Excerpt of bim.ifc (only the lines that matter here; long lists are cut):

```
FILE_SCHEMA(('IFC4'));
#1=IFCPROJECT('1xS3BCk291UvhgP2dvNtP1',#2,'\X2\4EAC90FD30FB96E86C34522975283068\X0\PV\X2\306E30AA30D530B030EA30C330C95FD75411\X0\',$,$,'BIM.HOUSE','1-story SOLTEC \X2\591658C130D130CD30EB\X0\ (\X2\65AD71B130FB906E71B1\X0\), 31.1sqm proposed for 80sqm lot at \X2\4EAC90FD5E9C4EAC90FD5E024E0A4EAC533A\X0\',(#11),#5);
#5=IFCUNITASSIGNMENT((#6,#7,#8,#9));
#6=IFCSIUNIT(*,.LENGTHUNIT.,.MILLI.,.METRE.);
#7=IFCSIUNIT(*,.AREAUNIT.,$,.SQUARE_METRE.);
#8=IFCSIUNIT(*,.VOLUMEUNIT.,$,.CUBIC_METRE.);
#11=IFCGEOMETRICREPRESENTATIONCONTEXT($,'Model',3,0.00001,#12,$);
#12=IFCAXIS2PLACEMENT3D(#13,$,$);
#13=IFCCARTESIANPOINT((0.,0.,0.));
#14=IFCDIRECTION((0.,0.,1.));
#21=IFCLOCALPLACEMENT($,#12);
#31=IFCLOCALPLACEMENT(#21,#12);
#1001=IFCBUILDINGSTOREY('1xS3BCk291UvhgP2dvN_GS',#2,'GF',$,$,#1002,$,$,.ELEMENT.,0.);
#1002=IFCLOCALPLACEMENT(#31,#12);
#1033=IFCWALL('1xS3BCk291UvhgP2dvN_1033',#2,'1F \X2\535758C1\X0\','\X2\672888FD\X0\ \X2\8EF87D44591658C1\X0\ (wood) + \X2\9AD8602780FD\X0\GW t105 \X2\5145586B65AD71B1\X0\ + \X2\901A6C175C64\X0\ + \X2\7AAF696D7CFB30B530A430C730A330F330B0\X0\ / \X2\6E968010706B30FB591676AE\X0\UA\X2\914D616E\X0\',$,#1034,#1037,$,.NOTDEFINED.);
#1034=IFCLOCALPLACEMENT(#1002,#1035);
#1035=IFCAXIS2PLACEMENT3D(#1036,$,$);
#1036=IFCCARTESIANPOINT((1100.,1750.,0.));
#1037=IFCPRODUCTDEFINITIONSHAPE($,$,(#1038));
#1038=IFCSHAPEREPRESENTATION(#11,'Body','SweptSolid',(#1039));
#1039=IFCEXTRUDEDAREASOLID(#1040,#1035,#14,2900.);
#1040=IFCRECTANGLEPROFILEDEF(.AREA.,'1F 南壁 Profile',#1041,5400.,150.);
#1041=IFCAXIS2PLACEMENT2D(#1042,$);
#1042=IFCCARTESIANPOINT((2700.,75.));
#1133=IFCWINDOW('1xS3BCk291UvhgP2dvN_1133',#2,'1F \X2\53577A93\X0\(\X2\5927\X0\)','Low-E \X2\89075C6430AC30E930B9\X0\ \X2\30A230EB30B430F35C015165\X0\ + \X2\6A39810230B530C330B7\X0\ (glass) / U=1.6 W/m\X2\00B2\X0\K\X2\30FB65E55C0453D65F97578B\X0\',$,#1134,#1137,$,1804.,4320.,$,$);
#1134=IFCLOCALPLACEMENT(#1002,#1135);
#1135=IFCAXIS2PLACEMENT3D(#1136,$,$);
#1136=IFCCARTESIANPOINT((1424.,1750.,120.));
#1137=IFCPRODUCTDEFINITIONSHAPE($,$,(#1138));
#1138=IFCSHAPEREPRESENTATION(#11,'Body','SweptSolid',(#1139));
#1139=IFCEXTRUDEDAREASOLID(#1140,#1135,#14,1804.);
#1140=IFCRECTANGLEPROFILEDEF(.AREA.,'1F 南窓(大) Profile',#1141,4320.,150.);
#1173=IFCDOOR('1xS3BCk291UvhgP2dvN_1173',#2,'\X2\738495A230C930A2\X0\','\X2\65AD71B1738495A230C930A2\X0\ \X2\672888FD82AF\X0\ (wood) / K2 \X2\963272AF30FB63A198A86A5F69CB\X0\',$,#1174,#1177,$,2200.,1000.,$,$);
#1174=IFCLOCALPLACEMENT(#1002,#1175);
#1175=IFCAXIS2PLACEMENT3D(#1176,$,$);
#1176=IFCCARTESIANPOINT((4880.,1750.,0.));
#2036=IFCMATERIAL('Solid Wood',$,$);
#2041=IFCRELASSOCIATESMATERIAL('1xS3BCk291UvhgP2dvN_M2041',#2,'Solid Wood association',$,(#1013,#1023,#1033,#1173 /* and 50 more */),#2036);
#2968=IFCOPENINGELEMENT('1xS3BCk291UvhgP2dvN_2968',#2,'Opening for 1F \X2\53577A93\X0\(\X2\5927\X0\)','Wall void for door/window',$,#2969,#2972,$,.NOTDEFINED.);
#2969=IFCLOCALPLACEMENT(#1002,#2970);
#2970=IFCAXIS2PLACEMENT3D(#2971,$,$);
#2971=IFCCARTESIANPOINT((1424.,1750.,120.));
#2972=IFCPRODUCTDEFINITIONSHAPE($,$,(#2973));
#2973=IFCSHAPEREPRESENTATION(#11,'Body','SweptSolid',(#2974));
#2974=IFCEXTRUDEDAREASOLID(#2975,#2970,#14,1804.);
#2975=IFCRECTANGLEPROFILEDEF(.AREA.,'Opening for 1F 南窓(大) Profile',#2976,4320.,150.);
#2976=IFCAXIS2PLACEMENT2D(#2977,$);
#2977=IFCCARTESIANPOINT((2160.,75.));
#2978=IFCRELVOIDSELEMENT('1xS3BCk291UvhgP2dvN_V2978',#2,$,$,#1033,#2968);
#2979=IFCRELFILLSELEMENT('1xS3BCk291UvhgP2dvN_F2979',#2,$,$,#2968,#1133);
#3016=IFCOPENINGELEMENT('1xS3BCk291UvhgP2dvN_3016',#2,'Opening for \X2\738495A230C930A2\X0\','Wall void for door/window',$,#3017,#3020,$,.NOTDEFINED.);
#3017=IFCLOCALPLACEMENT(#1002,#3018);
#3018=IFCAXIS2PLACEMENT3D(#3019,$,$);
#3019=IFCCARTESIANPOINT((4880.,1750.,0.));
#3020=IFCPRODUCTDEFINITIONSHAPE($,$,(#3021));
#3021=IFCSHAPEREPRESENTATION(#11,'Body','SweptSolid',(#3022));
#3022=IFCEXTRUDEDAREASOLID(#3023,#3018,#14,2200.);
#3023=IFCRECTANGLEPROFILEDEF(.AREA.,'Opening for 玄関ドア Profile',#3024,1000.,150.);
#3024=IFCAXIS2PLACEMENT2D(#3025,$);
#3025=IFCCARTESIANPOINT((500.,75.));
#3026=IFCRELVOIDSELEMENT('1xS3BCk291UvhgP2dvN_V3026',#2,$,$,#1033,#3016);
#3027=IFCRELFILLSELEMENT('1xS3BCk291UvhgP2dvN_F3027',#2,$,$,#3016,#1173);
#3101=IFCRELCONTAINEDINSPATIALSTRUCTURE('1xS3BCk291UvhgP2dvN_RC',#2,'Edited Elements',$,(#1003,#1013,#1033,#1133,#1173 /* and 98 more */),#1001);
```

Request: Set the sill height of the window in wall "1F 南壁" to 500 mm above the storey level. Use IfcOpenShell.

```python
import numpy as np
import ifcopenshell
import ifcopenshell.api.geometry
import ifcopenshell.geom
import ifcopenshell.util.element
import ifcopenshell.util.placement
import ifcopenshell.util.shape
import ifcopenshell.util.unit

model = ifcopenshell.open("bim.ifc")
unit_scale = ifcopenshell.util.unit.calculate_unit_scale(model)

window = model.by_guid("1xS3BCk291UvhgP2dvN_1133")
opening = window.FillsVoids[0].RelatingOpeningElement
storey = ifcopenshell.util.element.get_container(window, ifc_class="IfcBuildingStorey")
level = ifcopenshell.util.placement.get_local_placement(storey.ObjectPlacement)[2, 3]

# The opening's origin need not be at the sill, so measure its lowest point.
shape = ifcopenshell.geom.create_shape(ifcopenshell.geom.settings(), opening)
bottom = ifcopenshell.util.shape.get_shape_bottom_elevation(shape, shape.geometry) / unit_scale
dz = level + 0.5 / unit_scale - bottom

shift = np.array([0.0, 0.0, dz])
# The window is not placed relative to its opening, so move both.
for product in (opening, window):
    matrix = ifcopenshell.util.placement.get_local_placement(product.ObjectPlacement)
    matrix[:3, 3] += shift
    ifcopenshell.api.geometry.edit_object_placement(model, product=product, matrix=matrix, is_si=False)

print(f"moved by {dz * unit_scale:+.3f} m")

model.write("bim_updated.ifc")
```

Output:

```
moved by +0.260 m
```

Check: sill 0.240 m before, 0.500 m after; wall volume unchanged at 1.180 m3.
